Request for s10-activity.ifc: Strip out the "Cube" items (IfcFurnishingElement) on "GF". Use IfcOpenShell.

First a look at what the model holds.

```python
import ifcopenshell
import ifcopenshell.util.element

model = ifcopenshell.open("s10-activity.ifc")
print(model.schema)
storey = next(s for s in model.by_type("IfcBuildingStorey") if s.Name == "GF")
furniture = [e for e in ifcopenshell.util.element.get_decomposition(storey) if e.is_a("IfcFurnishingElement")]
seen = {}
for e in furniture:
    element_type = ifcopenshell.util.element.get_type(e)
    name = element_type.Name if element_type not in (None, e) else None
    seen[name] = seen.get(name, 0) + 1
for name, count in sorted(seen.items(), key=str):
    print(count, "x", name)
```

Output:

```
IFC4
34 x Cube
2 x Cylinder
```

```python
import ifcopenshell
import ifcopenshell.api.root
import ifcopenshell.util.element

model = ifcopenshell.open("s10-activity.ifc")

storey = next(s for s in model.by_type("IfcBuildingStorey") if s.Name == "GF")
furniture = [e for e in ifcopenshell.util.element.get_decomposition(storey) if e.is_a("IfcFurnishingElement")]
targets = [e for e in furniture if (t := ifcopenshell.util.element.get_type(e)) not in (None, e) and t.Name == "Cube"]

for e in targets:
    ifcopenshell.api.root.remove_product(model, product=e)
print(len(targets), "removed")

model.write("s10-activity_edited.ifc")
```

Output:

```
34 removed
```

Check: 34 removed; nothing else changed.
